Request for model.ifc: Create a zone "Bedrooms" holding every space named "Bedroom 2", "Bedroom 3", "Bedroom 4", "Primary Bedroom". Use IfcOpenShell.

First a look at what the model holds.

```python
import ifcopenshell

model = ifcopenshell.open("model.ifc")
print(model.schema)
seen = {}
for space in model.by_type("IfcSpace"):
    seen[space.LongName] = seen.get(space.LongName, 0) + 1
for name, count in sorted(seen.items(), key=str):
    print(count, "x", name)
print("zones:", [z.Name for z in model.by_type("IfcZone")][:20])
```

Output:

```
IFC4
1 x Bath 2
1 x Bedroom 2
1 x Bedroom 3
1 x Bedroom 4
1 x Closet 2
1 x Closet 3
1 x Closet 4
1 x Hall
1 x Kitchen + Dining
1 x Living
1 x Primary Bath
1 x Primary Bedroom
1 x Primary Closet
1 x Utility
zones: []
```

```python
import ifcopenshell
import ifcopenshell.api.group
import ifcopenshell.api.root

model = ifcopenshell.open("model.ifc")

names = {"Bedroom 2", "Bedroom 3", "Bedroom 4", "Primary Bedroom"}
spaces = [s for s in model.by_type("IfcSpace") if s.LongName in names]

zone = ifcopenshell.api.root.create_entity(model, ifc_class="IfcZone", name="Bedrooms")
ifcopenshell.api.group.assign_group(model, products=spaces, group=zone)
print(len(spaces), "spaces in", zone.Name)

model.write("model_updated.ifc")
```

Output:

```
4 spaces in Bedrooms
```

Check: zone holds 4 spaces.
